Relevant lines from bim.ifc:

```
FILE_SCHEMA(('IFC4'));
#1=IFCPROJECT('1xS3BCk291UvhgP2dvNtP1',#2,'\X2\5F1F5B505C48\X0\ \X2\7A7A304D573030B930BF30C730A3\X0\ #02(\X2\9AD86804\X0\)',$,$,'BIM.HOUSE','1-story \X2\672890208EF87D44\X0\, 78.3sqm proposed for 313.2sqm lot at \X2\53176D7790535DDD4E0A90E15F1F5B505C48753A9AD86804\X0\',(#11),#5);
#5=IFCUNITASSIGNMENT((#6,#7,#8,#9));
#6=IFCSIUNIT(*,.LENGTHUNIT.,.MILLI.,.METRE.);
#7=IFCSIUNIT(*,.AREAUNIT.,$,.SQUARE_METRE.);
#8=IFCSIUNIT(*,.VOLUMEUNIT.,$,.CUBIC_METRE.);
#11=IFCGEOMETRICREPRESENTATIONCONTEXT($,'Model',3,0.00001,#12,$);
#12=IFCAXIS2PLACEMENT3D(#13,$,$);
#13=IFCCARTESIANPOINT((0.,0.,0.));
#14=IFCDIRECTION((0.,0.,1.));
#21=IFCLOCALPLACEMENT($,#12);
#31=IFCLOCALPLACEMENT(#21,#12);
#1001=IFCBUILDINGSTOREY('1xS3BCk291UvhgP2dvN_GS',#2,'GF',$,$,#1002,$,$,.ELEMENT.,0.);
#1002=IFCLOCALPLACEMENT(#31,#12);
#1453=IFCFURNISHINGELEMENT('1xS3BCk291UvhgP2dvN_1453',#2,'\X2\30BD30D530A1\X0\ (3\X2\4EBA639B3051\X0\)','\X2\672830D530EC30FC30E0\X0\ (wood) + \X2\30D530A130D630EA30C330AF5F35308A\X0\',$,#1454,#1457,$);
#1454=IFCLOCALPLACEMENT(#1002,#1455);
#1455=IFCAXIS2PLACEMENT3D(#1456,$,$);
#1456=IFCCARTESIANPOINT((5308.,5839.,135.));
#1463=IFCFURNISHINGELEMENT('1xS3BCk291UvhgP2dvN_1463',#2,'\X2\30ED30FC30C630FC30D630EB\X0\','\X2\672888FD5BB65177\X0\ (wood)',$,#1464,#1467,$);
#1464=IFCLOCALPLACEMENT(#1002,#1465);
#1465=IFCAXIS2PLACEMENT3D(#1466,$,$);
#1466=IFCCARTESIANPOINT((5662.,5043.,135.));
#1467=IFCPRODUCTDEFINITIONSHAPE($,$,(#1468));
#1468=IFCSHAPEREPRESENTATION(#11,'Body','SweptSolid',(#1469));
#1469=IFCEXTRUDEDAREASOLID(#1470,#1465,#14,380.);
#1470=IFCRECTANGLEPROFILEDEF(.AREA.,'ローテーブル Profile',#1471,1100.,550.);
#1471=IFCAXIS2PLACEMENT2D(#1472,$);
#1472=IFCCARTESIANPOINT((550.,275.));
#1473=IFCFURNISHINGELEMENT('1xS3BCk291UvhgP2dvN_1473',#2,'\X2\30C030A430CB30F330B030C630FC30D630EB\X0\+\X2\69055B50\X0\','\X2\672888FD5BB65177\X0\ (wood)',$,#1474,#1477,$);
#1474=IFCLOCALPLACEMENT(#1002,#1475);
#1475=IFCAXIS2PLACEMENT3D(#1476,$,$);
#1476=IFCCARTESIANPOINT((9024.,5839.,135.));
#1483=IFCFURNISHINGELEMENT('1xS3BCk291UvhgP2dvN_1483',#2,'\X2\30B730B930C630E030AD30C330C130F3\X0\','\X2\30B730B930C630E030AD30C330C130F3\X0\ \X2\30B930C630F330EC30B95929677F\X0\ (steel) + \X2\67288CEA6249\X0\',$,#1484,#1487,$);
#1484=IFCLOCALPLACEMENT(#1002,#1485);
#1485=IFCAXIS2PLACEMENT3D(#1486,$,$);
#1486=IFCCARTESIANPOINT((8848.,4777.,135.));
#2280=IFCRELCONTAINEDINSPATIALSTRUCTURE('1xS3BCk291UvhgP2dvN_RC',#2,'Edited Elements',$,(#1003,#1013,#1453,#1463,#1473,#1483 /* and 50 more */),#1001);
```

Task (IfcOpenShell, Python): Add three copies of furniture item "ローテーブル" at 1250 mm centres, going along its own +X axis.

```python
import ifcopenshell
import ifcopenshell.api.geometry
import ifcopenshell.api.root
import ifcopenshell.util.element
import ifcopenshell.util.placement
import ifcopenshell.util.unit

model = ifcopenshell.open("bim.ifc")
unit_scale = ifcopenshell.util.unit.calculate_unit_scale(model)


def reuse_history(source, copy):
    """copy_class also copies each property set's owner history, people and application; keep the originals."""
    for rel in copy.IsDefinedBy:
        if rel.is_a("IfcRelDefinesByProperties") and (history := rel.RelatingPropertyDefinition.OwnerHistory):
            rel.RelatingPropertyDefinition.OwnerHistory = source.OwnerHistory
            ifcopenshell.util.element.remove_deep2(model, history)


source = model.by_guid("1xS3BCk291UvhgP2dvN_1463")
base = ifcopenshell.util.placement.get_local_placement(source.ObjectPlacement)
step = base[:3, 0] * 1.25 / unit_scale

for i in range(1, 4):
    copy = ifcopenshell.api.root.copy_class(model, product=source)
    copy.Representation = ifcopenshell.util.element.copy_deep(
        model, source.Representation, exclude=["IfcGeometricRepresentationContext", "IfcRepresentationMap"]
    )
    reuse_history(source, copy)
    matrix = base.copy()
    matrix[:3, 3] += i * step
    print("added at", matrix[:3, 3].round(3) + 0.0)
    ifcopenshell.api.geometry.edit_object_placement(model, product=copy, matrix=matrix, is_si=False)

model.write("bim_updated.ifc")
```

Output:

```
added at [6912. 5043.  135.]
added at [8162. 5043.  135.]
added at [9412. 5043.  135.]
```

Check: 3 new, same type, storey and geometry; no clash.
